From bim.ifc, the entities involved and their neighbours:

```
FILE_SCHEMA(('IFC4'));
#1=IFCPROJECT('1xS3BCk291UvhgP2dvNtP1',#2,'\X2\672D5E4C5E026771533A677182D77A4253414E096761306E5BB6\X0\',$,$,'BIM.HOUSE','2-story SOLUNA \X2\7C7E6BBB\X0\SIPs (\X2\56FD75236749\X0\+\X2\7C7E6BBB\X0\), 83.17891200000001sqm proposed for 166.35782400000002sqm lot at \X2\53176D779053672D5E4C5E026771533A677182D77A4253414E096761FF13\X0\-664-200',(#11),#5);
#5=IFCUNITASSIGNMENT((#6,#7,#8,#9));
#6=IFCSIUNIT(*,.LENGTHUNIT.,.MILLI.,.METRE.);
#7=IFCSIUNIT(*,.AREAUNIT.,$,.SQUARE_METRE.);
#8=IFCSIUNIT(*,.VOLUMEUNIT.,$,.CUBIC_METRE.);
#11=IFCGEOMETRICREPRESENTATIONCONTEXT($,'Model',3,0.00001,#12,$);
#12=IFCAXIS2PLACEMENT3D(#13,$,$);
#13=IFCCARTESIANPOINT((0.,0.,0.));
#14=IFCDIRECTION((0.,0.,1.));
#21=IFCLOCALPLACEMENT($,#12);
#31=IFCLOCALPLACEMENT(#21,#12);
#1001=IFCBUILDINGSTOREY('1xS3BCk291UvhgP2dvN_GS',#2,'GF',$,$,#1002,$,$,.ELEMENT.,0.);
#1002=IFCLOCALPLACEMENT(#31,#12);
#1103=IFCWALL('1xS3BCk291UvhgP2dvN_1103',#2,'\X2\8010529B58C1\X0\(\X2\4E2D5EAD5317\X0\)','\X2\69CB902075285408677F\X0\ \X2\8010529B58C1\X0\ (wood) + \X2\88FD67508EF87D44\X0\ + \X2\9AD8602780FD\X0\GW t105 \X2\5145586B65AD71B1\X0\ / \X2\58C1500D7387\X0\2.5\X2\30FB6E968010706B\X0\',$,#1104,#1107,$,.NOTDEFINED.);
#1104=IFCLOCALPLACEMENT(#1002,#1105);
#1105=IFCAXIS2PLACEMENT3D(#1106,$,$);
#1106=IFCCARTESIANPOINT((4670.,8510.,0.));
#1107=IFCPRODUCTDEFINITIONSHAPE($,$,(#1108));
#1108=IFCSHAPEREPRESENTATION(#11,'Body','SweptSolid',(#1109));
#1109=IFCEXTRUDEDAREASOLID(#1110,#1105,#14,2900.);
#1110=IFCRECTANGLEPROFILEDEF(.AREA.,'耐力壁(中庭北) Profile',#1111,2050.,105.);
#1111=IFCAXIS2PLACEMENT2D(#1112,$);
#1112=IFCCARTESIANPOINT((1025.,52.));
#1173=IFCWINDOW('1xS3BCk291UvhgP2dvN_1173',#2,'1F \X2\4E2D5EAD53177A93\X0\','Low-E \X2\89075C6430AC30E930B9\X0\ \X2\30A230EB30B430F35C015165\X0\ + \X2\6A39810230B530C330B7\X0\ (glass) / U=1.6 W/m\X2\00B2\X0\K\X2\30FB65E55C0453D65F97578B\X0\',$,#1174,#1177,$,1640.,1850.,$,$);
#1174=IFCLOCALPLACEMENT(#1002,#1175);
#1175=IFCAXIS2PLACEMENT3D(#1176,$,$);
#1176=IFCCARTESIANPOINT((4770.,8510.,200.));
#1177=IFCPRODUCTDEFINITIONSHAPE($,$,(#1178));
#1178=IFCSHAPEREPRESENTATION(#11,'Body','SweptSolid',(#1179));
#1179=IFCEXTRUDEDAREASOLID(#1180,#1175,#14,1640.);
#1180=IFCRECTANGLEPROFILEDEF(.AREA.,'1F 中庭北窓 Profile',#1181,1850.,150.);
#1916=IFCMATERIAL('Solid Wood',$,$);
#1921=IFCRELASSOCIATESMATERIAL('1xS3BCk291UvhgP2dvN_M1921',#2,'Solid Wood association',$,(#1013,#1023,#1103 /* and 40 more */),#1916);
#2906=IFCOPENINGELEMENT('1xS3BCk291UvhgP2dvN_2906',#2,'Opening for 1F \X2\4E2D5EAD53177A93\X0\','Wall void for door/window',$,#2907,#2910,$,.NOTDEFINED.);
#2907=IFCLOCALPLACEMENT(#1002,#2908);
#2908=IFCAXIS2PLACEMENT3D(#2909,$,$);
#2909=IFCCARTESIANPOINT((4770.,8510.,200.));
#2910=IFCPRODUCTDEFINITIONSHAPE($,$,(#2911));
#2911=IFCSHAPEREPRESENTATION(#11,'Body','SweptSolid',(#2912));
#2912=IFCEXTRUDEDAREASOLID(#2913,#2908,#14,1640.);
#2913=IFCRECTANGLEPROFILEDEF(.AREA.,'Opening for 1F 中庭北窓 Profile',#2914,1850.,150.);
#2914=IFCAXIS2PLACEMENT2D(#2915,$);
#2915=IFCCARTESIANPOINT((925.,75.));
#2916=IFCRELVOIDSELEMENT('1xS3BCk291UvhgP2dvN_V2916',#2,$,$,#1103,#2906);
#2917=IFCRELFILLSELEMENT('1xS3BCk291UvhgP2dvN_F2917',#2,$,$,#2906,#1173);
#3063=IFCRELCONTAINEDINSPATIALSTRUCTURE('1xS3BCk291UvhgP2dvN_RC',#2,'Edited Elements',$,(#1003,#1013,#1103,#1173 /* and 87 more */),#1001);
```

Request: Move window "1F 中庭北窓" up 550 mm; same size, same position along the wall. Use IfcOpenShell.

```python
import numpy as np
import ifcopenshell
import ifcopenshell.api.geometry
import ifcopenshell.util.placement
import ifcopenshell.util.unit

model = ifcopenshell.open("bim.ifc")
unit_scale = ifcopenshell.util.unit.calculate_unit_scale(model)

window = model.by_id(1173)
opening = window.FillsVoids[0].RelatingOpeningElement
dz = 0.55 / unit_scale

shift = np.array([0.0, 0.0, dz])
# The window is not placed relative to its opening, so move both.
for product in (opening, window):
    matrix = ifcopenshell.util.placement.get_local_placement(product.ObjectPlacement)
    matrix[:3, 3] += shift
    ifcopenshell.api.geometry.edit_object_placement(model, product=product, matrix=matrix, is_si=False)

print(f"moved by {dz * unit_scale:+.3f} m")

model.write("bim_rev.ifc")
```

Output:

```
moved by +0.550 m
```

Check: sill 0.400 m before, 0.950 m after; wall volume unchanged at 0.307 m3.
